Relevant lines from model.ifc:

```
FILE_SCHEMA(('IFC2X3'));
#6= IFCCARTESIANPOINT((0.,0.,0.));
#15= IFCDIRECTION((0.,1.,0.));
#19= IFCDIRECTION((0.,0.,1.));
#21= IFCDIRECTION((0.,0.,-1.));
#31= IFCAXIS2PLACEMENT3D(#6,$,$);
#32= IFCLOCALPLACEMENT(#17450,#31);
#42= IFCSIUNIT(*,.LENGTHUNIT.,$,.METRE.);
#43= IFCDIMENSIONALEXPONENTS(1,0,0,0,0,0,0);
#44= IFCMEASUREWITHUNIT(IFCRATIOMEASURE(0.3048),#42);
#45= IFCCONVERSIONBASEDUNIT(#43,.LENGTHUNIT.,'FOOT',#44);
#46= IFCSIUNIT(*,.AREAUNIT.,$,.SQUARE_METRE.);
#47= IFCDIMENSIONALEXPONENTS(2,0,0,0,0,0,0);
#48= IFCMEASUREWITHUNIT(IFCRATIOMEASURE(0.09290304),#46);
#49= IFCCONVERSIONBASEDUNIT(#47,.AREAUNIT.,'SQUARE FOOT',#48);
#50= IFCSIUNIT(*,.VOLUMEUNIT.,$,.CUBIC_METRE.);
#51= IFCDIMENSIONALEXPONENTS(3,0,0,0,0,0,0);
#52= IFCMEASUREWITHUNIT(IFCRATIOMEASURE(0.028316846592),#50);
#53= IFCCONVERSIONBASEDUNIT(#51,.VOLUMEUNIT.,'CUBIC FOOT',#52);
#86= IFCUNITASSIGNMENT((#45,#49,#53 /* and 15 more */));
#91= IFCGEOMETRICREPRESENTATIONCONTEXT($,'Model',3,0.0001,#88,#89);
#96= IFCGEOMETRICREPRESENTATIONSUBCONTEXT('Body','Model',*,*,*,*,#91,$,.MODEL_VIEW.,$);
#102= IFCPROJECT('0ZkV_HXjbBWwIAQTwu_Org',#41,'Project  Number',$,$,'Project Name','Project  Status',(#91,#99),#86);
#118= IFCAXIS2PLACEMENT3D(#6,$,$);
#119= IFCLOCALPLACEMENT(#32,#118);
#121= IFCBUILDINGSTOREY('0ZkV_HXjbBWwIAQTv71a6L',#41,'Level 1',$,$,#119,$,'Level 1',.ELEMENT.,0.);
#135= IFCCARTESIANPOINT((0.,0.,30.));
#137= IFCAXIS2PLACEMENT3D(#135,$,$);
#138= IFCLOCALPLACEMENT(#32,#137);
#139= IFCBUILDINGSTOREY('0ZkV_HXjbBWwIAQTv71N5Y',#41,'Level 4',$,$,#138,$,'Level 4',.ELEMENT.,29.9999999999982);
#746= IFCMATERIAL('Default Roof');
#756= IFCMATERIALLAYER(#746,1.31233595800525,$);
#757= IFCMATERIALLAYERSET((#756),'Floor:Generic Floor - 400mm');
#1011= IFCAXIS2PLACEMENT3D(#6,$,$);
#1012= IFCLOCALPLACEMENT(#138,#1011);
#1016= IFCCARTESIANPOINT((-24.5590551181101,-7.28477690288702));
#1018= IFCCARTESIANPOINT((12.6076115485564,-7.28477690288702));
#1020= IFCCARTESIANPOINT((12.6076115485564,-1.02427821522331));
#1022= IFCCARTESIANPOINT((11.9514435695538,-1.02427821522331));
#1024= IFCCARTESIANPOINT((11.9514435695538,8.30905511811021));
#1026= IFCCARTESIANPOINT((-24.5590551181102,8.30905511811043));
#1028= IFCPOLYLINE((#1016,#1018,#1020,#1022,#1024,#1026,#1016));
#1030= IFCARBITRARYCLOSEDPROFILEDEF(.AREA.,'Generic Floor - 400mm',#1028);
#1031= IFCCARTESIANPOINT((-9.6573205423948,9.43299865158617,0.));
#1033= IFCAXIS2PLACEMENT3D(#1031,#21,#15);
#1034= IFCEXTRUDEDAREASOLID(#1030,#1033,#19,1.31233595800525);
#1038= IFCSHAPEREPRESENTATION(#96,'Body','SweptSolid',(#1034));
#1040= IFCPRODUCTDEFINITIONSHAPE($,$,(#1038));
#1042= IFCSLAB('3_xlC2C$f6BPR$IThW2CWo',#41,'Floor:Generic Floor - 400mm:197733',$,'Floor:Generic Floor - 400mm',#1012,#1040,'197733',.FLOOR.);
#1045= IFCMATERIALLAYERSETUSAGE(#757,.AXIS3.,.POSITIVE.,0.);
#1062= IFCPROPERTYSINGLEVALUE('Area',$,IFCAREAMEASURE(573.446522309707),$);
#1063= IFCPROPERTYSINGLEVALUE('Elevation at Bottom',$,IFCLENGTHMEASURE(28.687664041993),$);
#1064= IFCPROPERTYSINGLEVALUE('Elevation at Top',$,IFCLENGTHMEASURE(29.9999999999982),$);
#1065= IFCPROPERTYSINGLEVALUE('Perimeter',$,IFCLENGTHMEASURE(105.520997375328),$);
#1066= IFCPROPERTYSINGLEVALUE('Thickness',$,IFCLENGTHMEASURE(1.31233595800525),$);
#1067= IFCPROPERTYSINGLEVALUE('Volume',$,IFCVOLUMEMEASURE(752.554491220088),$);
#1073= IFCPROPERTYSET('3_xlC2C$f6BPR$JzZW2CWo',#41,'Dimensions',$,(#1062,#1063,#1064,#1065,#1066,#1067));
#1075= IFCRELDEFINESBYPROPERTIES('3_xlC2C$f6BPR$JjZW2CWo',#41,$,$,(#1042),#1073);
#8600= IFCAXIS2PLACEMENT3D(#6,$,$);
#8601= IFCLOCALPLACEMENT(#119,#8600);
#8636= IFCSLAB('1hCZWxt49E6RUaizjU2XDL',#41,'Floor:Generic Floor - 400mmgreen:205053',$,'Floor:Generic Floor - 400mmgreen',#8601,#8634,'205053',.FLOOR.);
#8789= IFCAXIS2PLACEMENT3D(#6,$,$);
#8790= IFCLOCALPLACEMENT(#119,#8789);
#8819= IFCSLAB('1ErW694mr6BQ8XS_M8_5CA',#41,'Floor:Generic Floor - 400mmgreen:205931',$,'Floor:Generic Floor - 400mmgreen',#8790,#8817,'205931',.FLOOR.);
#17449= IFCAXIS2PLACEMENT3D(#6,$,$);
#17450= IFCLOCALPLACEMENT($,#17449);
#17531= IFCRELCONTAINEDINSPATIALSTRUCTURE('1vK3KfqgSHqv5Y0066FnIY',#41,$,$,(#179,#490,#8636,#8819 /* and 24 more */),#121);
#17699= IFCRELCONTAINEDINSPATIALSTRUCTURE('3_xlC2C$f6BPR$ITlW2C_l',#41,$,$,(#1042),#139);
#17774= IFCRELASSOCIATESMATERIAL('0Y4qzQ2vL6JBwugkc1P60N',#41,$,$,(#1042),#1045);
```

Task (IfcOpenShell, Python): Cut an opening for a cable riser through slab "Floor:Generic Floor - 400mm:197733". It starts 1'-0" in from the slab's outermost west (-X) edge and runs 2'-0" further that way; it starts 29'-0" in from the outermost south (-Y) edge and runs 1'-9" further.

```python
import numpy as np
import ifcopenshell
import ifcopenshell.api.feature
import ifcopenshell.api.geometry
import ifcopenshell.api.pset
import ifcopenshell.api.root
import ifcopenshell.geom
import ifcopenshell.util.element
import ifcopenshell.util.placement
import ifcopenshell.util.representation
import ifcopenshell.util.shape
import ifcopenshell.util.unit

model = ifcopenshell.open("model.ifc")
unit_scale = ifcopenshell.util.unit.calculate_unit_scale(model)
area_scale = ifcopenshell.util.unit.calculate_unit_scale(model, "AREAUNIT")
volume_scale = ifcopenshell.util.unit.calculate_unit_scale(model, "VOLUMEUNIT")
settings = ifcopenshell.geom.settings()


def volume(element):
    """Net volume in cubic metres, openings subtracted."""
    shape = ifcopenshell.geom.create_shape(settings, element)
    return ifcopenshell.util.shape.get_volume(shape.geometry)


slab = model.by_guid("3_xlC2C$f6BPR$IThW2CWo")
before = volume(slab)

# Extent in the slab's own axes, in metres. The edges named are its -X and -Y sides.
slab_shape = ifcopenshell.geom.create_shape(settings, slab)
vertices = ifcopenshell.util.shape.get_vertices(slab_shape.geometry)
x_min, y_min, bottom = vertices.min(axis=0)
top = vertices[:, 2].max()

opening = ifcopenshell.api.root.create_entity(model, ifc_class="IfcOpeningElement", name="Cable riser opening")
context = ifcopenshell.util.representation.get_context(model, "Model", "Body", "MODEL_VIEW")
width, depth = 0.6096, 0.5334
outline = [(0.0, 0.0), (width, 0.0), (width, depth), (0.0, depth), (0.0, 0.0)]
# Overshoot both faces by 50 mm so the cut is clean.
shape = ifcopenshell.api.geometry.add_slab_representation(
    model, context=context, depth=top - bottom + 0.1, polyline=outline
)
ifcopenshell.api.geometry.assign_representation(model, product=opening, representation=shape)

matrix = ifcopenshell.util.placement.get_local_placement(slab.ObjectPlacement)
matrix[:, 3] = matrix @ np.append(np.array([x_min + 0.3048, y_min + 8.8392, bottom - 0.05]) / unit_scale, 1.0)
ifcopenshell.api.geometry.edit_object_placement(model, product=opening, matrix=matrix, is_si=False)
ifcopenshell.api.feature.add_feature(model, feature=opening, element=slab)

after = volume(slab)

# Update the slab's stored quantities.
pset = model.by_id(ifcopenshell.util.element.get_pset(slab, "Dimensions", should_inherit=False)["id"])
ifcopenshell.api.pset.edit_pset(model, pset=pset, properties={
    "Area": model.create_entity("IfcAreaMeasure", after / (top - bottom) / area_scale),
    "Volume": model.create_entity("IfcVolumeMeasure", after / volume_scale),
})

print(f"slab volume {before:.3f} -> {after:.3f} m3")

model.write("model_v2.ifc")
```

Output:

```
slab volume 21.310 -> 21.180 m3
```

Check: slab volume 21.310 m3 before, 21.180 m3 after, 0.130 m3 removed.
